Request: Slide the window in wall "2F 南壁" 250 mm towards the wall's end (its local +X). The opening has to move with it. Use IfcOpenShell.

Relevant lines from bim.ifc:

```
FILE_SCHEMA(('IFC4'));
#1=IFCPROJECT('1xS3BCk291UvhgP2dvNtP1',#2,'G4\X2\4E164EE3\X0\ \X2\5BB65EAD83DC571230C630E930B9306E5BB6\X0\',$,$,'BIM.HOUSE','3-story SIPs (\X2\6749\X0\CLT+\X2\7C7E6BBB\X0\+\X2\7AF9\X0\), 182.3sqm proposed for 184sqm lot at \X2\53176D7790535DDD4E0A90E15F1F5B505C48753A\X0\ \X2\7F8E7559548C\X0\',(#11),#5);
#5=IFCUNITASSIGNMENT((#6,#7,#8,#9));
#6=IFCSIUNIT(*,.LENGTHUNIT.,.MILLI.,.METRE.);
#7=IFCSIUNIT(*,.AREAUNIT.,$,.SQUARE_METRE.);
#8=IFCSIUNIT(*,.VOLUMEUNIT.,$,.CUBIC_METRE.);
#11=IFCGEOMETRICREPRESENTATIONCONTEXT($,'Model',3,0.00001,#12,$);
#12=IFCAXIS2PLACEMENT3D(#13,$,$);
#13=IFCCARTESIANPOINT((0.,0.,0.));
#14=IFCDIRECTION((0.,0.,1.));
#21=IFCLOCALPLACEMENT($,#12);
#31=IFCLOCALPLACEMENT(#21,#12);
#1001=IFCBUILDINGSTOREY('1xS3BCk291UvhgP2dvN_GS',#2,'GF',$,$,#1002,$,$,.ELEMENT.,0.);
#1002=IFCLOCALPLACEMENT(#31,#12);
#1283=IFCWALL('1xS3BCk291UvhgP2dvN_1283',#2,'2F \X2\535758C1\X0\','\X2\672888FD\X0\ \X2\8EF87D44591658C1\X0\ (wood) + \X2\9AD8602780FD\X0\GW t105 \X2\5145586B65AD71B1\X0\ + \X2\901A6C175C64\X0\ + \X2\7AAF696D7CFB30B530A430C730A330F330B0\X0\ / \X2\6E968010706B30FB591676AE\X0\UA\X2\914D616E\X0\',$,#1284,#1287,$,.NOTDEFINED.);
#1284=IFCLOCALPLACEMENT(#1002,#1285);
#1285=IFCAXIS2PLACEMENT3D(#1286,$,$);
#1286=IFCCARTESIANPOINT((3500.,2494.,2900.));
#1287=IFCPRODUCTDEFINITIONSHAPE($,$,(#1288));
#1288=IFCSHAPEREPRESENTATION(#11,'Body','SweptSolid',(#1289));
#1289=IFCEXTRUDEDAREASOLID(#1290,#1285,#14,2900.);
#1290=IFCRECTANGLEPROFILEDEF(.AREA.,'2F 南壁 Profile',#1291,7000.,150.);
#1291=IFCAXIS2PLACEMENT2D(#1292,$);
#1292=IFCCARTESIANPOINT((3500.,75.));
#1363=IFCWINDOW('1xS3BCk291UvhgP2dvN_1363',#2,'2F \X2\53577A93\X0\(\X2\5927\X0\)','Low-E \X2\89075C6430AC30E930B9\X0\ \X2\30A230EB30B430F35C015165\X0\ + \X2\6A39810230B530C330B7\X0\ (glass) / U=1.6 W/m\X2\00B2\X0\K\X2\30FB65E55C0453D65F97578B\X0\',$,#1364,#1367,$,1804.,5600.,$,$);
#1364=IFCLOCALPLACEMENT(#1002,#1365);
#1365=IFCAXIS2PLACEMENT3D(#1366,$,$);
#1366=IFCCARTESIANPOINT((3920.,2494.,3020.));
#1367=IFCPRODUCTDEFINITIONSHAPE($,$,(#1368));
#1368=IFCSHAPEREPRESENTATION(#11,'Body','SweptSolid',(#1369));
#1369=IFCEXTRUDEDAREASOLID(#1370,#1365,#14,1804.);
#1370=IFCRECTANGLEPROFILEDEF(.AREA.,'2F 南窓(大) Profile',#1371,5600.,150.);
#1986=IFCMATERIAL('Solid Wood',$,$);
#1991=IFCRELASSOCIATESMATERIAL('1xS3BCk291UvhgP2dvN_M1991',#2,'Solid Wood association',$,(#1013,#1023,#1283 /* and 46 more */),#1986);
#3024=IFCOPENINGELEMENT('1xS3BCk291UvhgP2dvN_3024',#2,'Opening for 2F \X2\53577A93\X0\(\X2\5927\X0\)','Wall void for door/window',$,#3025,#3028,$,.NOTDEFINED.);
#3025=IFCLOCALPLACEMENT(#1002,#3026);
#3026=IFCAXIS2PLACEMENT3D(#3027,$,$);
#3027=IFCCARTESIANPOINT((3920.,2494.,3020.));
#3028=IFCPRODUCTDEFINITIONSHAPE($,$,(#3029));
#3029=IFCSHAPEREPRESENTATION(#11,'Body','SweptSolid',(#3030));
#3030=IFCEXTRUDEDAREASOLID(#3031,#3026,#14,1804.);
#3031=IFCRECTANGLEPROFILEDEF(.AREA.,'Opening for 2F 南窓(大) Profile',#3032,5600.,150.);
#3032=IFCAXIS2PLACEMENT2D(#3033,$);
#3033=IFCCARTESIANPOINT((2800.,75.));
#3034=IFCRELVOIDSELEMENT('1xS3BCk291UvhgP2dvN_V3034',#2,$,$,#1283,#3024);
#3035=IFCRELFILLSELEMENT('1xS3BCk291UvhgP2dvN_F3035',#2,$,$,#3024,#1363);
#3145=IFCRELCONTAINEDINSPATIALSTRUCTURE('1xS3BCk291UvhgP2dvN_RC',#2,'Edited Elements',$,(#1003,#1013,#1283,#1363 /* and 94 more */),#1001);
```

```python
import ifcopenshell
import ifcopenshell.api.geometry
import ifcopenshell.util.placement

model = ifcopenshell.open("bim.ifc")

window = model.by_guid("1xS3BCk291UvhgP2dvN_1363")
opening = window.FillsVoids[0].RelatingOpeningElement
wall = opening.VoidsElements[0].RelatingBuildingElement

wall_matrix = ifcopenshell.util.placement.get_local_placement(wall.ObjectPlacement)
shift = wall_matrix[:3, 0] * 250.0
before = ifcopenshell.util.placement.get_local_placement(window.ObjectPlacement)[:3, 3].copy()

# The window is not placed relative to its opening, so move both.
for product in (opening, window):
    matrix = ifcopenshell.util.placement.get_local_placement(product.ObjectPlacement)
    matrix[:3, 3] += shift
    ifcopenshell.api.geometry.edit_object_placement(model, product=product, matrix=matrix, is_si=False)

after = ifcopenshell.util.placement.get_local_placement(window.ObjectPlacement)[:3, 3]
print("window moved by", (after - before).round(3) + 0.0)

model.write("bim_edited.ifc")
```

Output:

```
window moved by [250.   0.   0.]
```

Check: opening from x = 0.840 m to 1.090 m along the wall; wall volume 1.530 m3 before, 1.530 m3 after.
